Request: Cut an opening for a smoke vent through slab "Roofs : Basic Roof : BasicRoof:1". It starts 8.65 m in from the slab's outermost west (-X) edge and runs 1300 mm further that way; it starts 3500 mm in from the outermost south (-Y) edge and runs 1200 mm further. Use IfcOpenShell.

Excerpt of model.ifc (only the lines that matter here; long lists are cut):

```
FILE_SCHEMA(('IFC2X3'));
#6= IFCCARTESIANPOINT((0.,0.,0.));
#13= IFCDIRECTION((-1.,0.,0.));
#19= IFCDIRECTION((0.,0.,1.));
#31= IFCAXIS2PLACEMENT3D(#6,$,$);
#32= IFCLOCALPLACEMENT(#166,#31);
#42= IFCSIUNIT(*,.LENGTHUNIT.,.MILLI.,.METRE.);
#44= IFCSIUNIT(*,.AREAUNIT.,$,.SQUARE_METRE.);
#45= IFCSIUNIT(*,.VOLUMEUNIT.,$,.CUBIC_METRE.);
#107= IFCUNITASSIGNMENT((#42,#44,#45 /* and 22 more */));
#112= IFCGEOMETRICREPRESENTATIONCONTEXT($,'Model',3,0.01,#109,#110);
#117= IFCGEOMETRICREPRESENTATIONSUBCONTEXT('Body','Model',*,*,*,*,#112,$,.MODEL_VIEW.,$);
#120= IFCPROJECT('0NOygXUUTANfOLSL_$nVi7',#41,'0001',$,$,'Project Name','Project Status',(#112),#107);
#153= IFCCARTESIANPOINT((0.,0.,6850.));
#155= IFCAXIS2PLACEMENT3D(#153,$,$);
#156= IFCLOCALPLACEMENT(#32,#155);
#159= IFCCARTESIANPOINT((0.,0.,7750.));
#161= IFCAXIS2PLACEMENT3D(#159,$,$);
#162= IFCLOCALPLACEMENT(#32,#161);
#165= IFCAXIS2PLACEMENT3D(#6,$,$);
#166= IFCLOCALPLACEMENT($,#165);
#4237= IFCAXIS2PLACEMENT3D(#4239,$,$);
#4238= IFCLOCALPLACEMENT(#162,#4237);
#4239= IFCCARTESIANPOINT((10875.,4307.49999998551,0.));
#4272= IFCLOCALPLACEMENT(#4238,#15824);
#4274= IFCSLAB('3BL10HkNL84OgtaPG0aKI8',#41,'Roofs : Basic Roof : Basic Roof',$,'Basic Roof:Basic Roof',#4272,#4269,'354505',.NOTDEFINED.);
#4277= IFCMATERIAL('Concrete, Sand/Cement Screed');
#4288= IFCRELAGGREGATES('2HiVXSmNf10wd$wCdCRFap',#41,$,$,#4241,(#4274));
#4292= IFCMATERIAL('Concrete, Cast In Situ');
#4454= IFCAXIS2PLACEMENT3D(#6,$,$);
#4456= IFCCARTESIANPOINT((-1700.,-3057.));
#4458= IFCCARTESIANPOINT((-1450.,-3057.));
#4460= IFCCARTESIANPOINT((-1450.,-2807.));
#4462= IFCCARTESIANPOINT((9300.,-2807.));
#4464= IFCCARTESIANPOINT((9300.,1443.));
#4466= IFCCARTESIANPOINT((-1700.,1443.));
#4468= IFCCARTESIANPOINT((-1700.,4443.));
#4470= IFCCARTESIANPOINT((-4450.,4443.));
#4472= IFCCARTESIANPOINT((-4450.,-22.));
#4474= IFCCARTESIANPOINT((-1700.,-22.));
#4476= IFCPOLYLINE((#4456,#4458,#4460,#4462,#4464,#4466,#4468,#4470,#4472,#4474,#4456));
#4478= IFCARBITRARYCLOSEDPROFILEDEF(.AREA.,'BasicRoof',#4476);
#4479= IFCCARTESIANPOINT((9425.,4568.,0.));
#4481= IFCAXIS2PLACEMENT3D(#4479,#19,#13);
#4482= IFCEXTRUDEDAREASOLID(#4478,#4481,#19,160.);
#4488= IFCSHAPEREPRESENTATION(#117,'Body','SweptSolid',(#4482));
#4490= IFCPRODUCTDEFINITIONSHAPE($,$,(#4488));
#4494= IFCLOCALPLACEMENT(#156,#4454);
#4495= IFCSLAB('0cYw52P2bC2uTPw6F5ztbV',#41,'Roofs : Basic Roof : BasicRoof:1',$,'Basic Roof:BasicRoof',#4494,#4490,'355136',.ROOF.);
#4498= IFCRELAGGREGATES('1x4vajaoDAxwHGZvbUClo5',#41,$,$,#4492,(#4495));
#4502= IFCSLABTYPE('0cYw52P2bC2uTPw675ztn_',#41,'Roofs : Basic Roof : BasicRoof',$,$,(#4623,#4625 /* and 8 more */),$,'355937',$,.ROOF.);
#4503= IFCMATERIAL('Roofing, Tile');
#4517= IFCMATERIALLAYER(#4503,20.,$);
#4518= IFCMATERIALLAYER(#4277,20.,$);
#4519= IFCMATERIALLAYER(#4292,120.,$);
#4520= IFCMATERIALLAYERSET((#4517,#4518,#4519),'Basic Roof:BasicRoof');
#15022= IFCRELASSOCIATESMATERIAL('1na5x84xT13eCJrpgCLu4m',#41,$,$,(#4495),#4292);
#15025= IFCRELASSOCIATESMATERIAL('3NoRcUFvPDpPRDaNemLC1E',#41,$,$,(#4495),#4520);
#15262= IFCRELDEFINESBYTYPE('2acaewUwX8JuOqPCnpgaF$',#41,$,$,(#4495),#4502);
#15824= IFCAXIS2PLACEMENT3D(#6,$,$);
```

```python
import numpy as np
import ifcopenshell
import ifcopenshell.api.feature
import ifcopenshell.api.geometry
import ifcopenshell.api.root
import ifcopenshell.geom
import ifcopenshell.util.placement
import ifcopenshell.util.representation
import ifcopenshell.util.shape
import ifcopenshell.util.unit

model = ifcopenshell.open("model.ifc")
unit_scale = ifcopenshell.util.unit.calculate_unit_scale(model)
settings = ifcopenshell.geom.settings()


def volume(element):
    """Net volume in cubic metres, openings subtracted."""
    shape = ifcopenshell.geom.create_shape(settings, element)
    return ifcopenshell.util.shape.get_volume(shape.geometry)


slab = model.by_guid("0cYw52P2bC2uTPw6F5ztbV")
before = volume(slab)

# Extent in the slab's own axes, in metres. The edges named are its -X and -Y sides.
slab_shape = ifcopenshell.geom.create_shape(settings, slab)
vertices = ifcopenshell.util.shape.get_vertices(slab_shape.geometry)
x_min, y_min, bottom = vertices.min(axis=0)
top = vertices[:, 2].max()

opening = ifcopenshell.api.root.create_entity(model, ifc_class="IfcOpeningElement", name="Smoke vent opening")
context = ifcopenshell.util.representation.get_context(model, "Model", "Body", "MODEL_VIEW")
width, depth = 1.3, 1.2
outline = [(0.0, 0.0), (width, 0.0), (width, depth), (0.0, depth), (0.0, 0.0)]
# Overshoot both faces by 50 mm so the cut is clean.
shape = ifcopenshell.api.geometry.add_slab_representation(
    model, context=context, depth=top - bottom + 0.1, polyline=outline
)
ifcopenshell.api.geometry.assign_representation(model, product=opening, representation=shape)

matrix = ifcopenshell.util.placement.get_local_placement(slab.ObjectPlacement)
matrix[:, 3] = matrix @ np.append(np.array([x_min + 8.65, y_min + 3.5, bottom - 0.05]) / unit_scale, 1.0)
ifcopenshell.api.geometry.edit_object_placement(model, product=opening, matrix=matrix, is_si=False)
ifcopenshell.api.feature.add_feature(model, feature=opening, element=slab)

after = volume(slab)

print(f"slab volume {before:.3f} -> {after:.3f} m3")

model.write("model_v2.ifc")
```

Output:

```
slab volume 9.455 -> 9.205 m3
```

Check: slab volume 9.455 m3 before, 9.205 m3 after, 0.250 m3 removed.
